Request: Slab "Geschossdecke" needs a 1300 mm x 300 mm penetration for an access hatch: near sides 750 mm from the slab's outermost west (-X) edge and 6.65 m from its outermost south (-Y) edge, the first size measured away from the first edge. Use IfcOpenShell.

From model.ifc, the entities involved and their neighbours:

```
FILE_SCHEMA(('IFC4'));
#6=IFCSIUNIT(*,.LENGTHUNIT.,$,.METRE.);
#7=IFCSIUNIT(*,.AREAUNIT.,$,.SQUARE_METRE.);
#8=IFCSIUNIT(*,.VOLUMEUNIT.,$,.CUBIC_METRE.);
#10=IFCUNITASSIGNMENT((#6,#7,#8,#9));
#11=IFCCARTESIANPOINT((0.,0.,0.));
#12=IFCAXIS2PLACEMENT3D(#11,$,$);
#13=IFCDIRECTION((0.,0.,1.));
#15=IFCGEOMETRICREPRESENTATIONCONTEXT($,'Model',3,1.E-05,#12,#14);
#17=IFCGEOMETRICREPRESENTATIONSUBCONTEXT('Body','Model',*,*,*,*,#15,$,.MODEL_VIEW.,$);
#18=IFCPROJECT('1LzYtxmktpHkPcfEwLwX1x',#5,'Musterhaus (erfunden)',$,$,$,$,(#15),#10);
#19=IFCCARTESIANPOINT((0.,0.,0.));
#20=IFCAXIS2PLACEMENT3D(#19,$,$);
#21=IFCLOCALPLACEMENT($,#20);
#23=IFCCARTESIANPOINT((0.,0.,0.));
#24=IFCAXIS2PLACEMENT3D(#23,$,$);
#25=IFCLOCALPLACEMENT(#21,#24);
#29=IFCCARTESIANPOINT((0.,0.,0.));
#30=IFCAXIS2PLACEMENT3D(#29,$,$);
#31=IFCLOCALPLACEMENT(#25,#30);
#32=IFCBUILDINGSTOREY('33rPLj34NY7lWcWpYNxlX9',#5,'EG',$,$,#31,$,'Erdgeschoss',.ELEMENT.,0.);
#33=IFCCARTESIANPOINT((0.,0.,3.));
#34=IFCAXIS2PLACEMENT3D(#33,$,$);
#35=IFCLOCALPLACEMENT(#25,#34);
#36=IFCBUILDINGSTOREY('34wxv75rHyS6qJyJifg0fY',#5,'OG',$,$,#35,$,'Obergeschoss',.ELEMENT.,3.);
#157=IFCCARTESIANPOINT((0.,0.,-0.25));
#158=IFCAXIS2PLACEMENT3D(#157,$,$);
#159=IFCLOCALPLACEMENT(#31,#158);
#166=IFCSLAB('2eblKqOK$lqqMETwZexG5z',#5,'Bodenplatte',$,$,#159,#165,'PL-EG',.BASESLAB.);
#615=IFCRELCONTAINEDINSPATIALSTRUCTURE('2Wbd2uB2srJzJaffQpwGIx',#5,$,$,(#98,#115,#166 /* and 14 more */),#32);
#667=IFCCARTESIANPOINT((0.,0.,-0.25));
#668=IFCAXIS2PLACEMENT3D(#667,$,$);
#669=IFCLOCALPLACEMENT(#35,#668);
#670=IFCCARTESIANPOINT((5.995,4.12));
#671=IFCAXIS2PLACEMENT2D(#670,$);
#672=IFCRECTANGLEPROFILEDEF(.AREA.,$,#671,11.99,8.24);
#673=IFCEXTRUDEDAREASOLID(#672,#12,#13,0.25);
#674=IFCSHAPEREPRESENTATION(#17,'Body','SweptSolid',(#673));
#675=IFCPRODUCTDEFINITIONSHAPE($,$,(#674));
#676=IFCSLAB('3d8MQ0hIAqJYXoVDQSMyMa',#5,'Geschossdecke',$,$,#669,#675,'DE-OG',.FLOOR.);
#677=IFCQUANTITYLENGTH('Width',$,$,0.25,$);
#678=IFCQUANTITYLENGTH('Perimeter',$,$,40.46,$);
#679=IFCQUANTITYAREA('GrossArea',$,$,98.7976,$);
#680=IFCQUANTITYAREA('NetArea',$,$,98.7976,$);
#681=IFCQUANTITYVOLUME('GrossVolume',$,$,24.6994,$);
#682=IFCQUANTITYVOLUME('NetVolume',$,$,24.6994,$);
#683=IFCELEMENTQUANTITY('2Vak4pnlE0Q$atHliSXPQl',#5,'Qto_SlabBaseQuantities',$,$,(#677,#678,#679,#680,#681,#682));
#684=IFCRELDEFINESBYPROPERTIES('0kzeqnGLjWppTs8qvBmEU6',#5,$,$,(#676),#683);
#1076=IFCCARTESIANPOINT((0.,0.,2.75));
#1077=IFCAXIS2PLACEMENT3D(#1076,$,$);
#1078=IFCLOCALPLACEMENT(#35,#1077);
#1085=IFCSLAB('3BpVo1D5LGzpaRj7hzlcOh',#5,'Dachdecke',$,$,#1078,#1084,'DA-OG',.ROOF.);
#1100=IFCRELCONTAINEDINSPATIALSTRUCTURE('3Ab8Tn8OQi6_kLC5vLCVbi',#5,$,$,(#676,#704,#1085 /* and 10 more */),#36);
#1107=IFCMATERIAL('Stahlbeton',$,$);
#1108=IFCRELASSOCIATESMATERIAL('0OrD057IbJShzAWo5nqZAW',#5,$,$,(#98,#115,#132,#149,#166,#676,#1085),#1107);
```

```python
import numpy as np
import ifcopenshell
import ifcopenshell.api.feature
import ifcopenshell.api.geometry
import ifcopenshell.api.pset
import ifcopenshell.api.root
import ifcopenshell.geom
import ifcopenshell.util.element
import ifcopenshell.util.placement
import ifcopenshell.util.representation
import ifcopenshell.util.shape
import ifcopenshell.util.unit

model = ifcopenshell.open("model.ifc")
unit_scale = ifcopenshell.util.unit.calculate_unit_scale(model)
area_scale = ifcopenshell.util.unit.calculate_unit_scale(model, "AREAUNIT")
volume_scale = ifcopenshell.util.unit.calculate_unit_scale(model, "VOLUMEUNIT")
settings = ifcopenshell.geom.settings()


def volume(element):
    """Net volume in cubic metres, openings subtracted."""
    shape = ifcopenshell.geom.create_shape(settings, element)
    return ifcopenshell.util.shape.get_volume(shape.geometry)


slab = model.by_guid("3d8MQ0hIAqJYXoVDQSMyMa")
before = volume(slab)

# Extent in the slab's own axes, in metres. The edges named are its -X and -Y sides.
slab_shape = ifcopenshell.geom.create_shape(settings, slab)
vertices = ifcopenshell.util.shape.get_vertices(slab_shape.geometry)
x_min, y_min, bottom = vertices.min(axis=0)
top = vertices[:, 2].max()

opening = ifcopenshell.api.root.create_entity(model, ifc_class="IfcOpeningElement", name="Access hatch opening", predefined_type="OPENING")
context = ifcopenshell.util.representation.get_context(model, "Model", "Body", "MODEL_VIEW")
width, depth = 1.3, 0.3
outline = [(0.0, 0.0), (width, 0.0), (width, depth), (0.0, depth), (0.0, 0.0)]
# Overshoot both faces by 50 mm so the cut is clean.
shape = ifcopenshell.api.geometry.add_slab_representation(
    model, context=context, depth=top - bottom + 0.1, polyline=outline
)
ifcopenshell.api.geometry.assign_representation(model, product=opening, representation=shape)

matrix = ifcopenshell.util.placement.get_local_placement(slab.ObjectPlacement)
matrix[:, 3] = matrix @ np.append(np.array([x_min + 0.75, y_min + 6.65, bottom - 0.05]) / unit_scale, 1.0)
ifcopenshell.api.geometry.edit_object_placement(model, product=opening, matrix=matrix, is_si=False)
ifcopenshell.api.feature.add_feature(model, feature=opening, element=slab)

after = volume(slab)

# Update the slab's stored quantities.
qto = model.by_id(ifcopenshell.util.element.get_pset(slab, "Qto_SlabBaseQuantities", should_inherit=False)["id"])
ifcopenshell.api.pset.edit_qto(model, qto=qto, properties={
    "NetArea": after / (top - bottom) / area_scale,
    "NetVolume": after / volume_scale,
})

print(f"slab volume {before:.3f} -> {after:.3f} m3")

model.write("model_rev.ifc")
```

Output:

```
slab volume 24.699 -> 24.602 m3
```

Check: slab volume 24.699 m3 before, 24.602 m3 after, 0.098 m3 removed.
